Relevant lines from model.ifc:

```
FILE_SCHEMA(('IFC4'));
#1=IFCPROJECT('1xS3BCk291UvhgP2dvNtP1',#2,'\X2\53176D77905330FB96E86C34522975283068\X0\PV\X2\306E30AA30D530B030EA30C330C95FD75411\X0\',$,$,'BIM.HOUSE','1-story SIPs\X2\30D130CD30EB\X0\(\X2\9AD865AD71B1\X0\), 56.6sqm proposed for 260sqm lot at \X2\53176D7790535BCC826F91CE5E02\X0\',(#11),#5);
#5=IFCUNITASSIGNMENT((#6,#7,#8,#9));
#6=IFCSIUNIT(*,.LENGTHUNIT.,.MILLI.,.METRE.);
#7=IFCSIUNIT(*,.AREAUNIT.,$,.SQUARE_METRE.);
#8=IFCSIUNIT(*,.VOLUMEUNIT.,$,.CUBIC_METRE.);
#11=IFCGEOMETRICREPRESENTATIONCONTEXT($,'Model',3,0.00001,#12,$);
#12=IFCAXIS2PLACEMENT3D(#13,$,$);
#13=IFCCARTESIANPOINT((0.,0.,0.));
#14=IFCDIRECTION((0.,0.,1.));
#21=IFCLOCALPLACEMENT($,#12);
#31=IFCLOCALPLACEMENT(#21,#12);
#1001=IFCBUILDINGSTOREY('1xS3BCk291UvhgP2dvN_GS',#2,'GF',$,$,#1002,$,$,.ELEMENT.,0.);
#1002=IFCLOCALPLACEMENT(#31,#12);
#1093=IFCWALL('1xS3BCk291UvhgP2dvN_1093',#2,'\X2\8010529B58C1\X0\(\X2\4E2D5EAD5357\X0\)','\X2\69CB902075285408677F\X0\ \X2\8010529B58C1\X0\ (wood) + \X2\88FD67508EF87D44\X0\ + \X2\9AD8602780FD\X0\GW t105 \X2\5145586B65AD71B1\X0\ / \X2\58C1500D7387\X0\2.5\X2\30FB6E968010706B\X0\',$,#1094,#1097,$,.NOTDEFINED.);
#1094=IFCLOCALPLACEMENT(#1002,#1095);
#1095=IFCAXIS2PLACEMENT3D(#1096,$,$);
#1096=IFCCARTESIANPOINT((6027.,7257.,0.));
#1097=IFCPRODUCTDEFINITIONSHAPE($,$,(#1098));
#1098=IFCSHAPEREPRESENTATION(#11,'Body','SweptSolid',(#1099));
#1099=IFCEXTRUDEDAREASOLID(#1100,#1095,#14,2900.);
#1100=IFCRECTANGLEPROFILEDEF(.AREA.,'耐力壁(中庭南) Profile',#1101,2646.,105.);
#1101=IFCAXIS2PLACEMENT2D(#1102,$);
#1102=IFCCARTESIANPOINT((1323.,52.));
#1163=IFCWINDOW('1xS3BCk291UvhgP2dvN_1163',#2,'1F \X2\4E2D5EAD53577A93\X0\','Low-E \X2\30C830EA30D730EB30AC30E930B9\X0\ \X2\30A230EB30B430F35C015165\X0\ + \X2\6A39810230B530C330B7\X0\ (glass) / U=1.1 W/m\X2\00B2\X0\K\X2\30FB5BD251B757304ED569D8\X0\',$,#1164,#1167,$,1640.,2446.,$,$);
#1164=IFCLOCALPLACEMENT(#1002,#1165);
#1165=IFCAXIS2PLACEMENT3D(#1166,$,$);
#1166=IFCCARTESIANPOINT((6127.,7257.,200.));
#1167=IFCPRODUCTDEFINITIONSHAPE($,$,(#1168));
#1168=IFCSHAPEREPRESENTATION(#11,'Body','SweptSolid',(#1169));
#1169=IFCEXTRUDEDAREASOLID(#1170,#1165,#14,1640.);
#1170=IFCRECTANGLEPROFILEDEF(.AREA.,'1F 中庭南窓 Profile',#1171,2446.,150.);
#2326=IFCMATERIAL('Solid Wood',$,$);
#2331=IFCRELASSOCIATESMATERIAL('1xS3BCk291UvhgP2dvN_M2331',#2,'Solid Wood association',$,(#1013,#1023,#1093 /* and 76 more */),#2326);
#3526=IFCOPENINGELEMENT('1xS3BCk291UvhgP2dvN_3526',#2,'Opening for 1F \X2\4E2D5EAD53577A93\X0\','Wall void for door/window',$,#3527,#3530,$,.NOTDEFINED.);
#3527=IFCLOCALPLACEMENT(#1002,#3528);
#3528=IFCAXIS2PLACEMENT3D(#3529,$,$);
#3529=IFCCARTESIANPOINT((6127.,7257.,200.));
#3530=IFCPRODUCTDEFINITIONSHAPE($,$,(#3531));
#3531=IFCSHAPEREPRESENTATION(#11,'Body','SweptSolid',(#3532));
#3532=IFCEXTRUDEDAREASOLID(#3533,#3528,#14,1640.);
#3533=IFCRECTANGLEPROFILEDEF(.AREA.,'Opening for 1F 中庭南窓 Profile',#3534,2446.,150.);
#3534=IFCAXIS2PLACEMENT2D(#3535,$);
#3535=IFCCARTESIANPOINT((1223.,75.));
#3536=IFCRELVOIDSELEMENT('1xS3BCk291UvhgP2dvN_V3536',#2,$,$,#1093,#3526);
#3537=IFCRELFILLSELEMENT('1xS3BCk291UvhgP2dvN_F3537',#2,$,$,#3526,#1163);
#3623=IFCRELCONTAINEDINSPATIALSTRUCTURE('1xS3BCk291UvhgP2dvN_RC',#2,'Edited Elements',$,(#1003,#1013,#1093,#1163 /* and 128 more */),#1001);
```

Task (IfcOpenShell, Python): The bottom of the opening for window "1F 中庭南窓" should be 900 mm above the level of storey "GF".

```python
import numpy as np
import ifcopenshell
import ifcopenshell.api.geometry
import ifcopenshell.geom
import ifcopenshell.util.element
import ifcopenshell.util.placement
import ifcopenshell.util.shape
import ifcopenshell.util.unit

model = ifcopenshell.open("model.ifc")
unit_scale = ifcopenshell.util.unit.calculate_unit_scale(model)

window = model.by_guid("1xS3BCk291UvhgP2dvN_1163")
opening = window.FillsVoids[0].RelatingOpeningElement
storey = ifcopenshell.util.element.get_container(window, ifc_class="IfcBuildingStorey")
level = ifcopenshell.util.placement.get_local_placement(storey.ObjectPlacement)[2, 3]

# The opening's origin need not be at the sill, so measure its lowest point.
shape = ifcopenshell.geom.create_shape(ifcopenshell.geom.settings(), opening)
bottom = ifcopenshell.util.shape.get_shape_bottom_elevation(shape, shape.geometry) / unit_scale
dz = level + 0.9 / unit_scale - bottom

shift = np.array([0.0, 0.0, dz])
# The window is not placed relative to its opening, so move both.
for product in (opening, window):
    matrix = ifcopenshell.util.placement.get_local_placement(product.ObjectPlacement)
    matrix[:3, 3] += shift
    ifcopenshell.api.geometry.edit_object_placement(model, product=product, matrix=matrix, is_si=False)

print(f"moved by {dz * unit_scale:+.3f} m")

model.write("model_updated.ifc")
```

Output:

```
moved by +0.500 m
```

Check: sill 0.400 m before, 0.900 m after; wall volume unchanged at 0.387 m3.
